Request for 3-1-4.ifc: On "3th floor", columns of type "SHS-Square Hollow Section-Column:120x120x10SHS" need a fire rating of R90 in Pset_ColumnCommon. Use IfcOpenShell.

First a look at what the model holds.

```python
import ifcopenshell
import ifcopenshell.util.element

model = ifcopenshell.open("3-1-4.ifc")
print(model.schema)
storey = next(s for s in model.by_type("IfcBuildingStorey") if s.Name == "3th floor")
columns = [e for e in ifcopenshell.util.element.get_decomposition(storey) if e.is_a("IfcColumn")]
seen = {}
for e in columns:
    element_type = ifcopenshell.util.element.get_type(e)
    key = (element_type.Name if element_type != e and element_type else None, ifcopenshell.util.element.get_pset(e, "Pset_ColumnCommon", "FireRating"))
    seen[key] = seen.get(key, 0) + 1
for (name, value), count in sorted(seen.items(), key=str):
    print(count, "x", name, "|", value)
```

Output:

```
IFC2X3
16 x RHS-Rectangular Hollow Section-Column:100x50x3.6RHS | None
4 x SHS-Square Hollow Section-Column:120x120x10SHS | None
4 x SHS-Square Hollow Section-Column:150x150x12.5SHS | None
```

```python
import ifcopenshell
import ifcopenshell.api.pset
import ifcopenshell.util.element

model = ifcopenshell.open("3-1-4.ifc")

storey = next(s for s in model.by_type("IfcBuildingStorey") if s.Name == "3th floor")
columns = [e for e in ifcopenshell.util.element.get_decomposition(storey) if e.is_a("IfcColumn")]

count = 0
for e in columns:
    element_type = ifcopenshell.util.element.get_type(e)
    if element_type in (None, e) or element_type.Name != "SHS-Square Hollow Section-Column:120x120x10SHS":
        continue
    # add_pset returns the element's existing set when there is one.
    pset = ifcopenshell.api.pset.add_pset(model, product=e, name="Pset_ColumnCommon")
    ifcopenshell.api.pset.edit_pset(model, pset=pset, properties={"FireRating": "R90"})
    count += 1

print(count, "columns updated")

model.write("3-1-4_updated.ifc")
```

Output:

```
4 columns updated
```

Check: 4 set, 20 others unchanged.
